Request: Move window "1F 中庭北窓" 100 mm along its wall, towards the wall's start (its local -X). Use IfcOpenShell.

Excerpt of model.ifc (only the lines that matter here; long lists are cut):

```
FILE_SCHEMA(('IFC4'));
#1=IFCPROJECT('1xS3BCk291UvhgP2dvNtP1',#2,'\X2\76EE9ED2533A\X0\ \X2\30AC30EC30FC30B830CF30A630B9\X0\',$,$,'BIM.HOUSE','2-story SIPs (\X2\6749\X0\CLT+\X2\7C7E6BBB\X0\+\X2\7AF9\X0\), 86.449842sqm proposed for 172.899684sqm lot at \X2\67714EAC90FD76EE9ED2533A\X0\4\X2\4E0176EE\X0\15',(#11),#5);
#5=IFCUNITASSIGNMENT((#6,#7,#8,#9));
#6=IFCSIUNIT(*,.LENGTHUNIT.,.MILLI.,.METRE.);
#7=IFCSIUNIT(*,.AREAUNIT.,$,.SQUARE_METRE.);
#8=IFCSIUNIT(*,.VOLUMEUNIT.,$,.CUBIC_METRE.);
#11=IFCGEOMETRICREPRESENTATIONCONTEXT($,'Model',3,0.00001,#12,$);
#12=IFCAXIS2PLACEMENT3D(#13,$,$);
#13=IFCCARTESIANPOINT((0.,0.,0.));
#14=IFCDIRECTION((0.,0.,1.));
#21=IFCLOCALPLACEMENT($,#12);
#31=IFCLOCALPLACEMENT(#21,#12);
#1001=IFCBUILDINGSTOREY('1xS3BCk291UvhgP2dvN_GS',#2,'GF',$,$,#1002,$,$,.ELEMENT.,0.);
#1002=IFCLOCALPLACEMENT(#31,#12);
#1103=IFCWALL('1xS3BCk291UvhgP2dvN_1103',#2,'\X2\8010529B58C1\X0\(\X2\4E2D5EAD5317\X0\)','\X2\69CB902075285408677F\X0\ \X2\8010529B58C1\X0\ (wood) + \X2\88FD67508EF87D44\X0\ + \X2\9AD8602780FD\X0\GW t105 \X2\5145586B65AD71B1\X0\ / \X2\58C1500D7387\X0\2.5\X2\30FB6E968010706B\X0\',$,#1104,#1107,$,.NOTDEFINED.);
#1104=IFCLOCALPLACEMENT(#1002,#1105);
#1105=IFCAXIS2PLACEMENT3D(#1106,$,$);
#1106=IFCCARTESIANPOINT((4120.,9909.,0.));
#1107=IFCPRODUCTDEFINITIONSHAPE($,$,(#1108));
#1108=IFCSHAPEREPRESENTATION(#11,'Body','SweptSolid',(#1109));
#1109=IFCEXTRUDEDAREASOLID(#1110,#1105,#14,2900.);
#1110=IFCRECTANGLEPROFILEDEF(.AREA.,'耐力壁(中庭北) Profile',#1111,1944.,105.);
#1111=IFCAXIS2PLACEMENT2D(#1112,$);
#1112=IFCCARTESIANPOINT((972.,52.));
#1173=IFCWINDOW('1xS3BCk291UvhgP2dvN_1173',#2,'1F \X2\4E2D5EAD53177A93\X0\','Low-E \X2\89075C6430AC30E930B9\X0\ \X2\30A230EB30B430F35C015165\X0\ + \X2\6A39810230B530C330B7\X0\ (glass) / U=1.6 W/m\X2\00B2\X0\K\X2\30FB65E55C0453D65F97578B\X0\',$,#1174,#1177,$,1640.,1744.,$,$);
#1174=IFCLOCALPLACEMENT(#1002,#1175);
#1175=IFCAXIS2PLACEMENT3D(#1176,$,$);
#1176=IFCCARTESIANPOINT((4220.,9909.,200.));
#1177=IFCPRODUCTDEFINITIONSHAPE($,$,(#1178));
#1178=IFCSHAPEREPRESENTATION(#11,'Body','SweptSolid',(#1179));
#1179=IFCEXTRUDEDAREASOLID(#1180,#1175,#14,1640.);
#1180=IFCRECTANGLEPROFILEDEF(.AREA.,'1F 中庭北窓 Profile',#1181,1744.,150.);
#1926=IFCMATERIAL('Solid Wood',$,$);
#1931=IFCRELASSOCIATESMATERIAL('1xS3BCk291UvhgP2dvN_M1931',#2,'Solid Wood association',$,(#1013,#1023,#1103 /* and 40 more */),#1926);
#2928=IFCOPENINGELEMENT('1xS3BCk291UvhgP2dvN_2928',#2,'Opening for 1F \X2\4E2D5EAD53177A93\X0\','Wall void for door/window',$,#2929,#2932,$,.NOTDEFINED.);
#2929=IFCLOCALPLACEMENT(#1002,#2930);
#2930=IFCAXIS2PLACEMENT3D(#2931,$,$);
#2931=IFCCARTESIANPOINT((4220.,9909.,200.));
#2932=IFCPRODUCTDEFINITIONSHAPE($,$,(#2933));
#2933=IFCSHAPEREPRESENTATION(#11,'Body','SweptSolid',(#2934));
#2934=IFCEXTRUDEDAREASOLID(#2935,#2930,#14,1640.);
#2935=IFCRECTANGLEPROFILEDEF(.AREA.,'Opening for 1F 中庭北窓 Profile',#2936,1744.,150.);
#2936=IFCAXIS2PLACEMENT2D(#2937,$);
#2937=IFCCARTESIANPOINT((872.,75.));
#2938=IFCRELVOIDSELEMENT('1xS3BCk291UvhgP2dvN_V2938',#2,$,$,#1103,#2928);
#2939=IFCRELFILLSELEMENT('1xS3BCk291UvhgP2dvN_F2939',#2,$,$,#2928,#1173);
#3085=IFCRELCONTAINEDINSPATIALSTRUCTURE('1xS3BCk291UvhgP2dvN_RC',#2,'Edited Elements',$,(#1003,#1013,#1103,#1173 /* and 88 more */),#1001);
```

```python
import ifcopenshell
import ifcopenshell.api.geometry
import ifcopenshell.util.placement
import ifcopenshell.util.unit

model = ifcopenshell.open("model.ifc")
unit_scale = ifcopenshell.util.unit.calculate_unit_scale(model)

window = model.by_guid("1xS3BCk291UvhgP2dvN_1173")
opening = window.FillsVoids[0].RelatingOpeningElement
wall = opening.VoidsElements[0].RelatingBuildingElement

wall_matrix = ifcopenshell.util.placement.get_local_placement(wall.ObjectPlacement)
shift = wall_matrix[:3, 0] * -0.1 / unit_scale
before = ifcopenshell.util.placement.get_local_placement(window.ObjectPlacement)[:3, 3].copy()

# The window is not placed relative to its opening, so move both.
for product in (opening, window):
    matrix = ifcopenshell.util.placement.get_local_placement(product.ObjectPlacement)
    matrix[:3, 3] += shift
    ifcopenshell.api.geometry.edit_object_placement(model, product=product, matrix=matrix, is_si=False)

after = ifcopenshell.util.placement.get_local_placement(window.ObjectPlacement)[:3, 3]
print("window moved by", (after - before).round(3) + 0.0)

model.write("model_updated.ifc")
```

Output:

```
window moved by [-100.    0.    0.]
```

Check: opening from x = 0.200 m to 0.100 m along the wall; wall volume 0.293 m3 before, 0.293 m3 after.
